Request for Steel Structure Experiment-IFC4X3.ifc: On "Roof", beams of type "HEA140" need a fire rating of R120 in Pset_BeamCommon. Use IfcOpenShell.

First a look at what the model holds.

```python
import ifcopenshell
import ifcopenshell.util.element

model = ifcopenshell.open("Steel Structure Experiment-IFC4X3.ifc")
print(model.schema)
storey = next(s for s in model.by_type("IfcBuildingStorey") if s.Name == "Roof")
beams = [e for e in ifcopenshell.util.element.get_decomposition(storey) if e.is_a("IfcBeam")]
seen = {}
for e in beams:
    element_type = ifcopenshell.util.element.get_type(e)
    key = (element_type.Name if element_type != e and element_type else None, ifcopenshell.util.element.get_pset(e, "Pset_BeamCommon", "FireRating"))
    seen[key] = seen.get(key, 0) + 1
for (name, value), count in sorted(seen.items(), key=str):
    print(count, "x", name, "|", value)
```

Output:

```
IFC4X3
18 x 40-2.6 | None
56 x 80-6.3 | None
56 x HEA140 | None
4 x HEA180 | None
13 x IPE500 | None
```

```python
import ifcopenshell
import ifcopenshell.api.pset
import ifcopenshell.util.element

model = ifcopenshell.open("Steel Structure Experiment-IFC4X3.ifc")

storey = next(s for s in model.by_type("IfcBuildingStorey") if s.Name == "Roof")
beams = [e for e in ifcopenshell.util.element.get_decomposition(storey) if e.is_a("IfcBeam")]

count = 0
for e in beams:
    element_type = ifcopenshell.util.element.get_type(e)
    if element_type in (None, e) or element_type.Name != "HEA140":
        continue
    # add_pset returns the element's existing set when there is one.
    pset = ifcopenshell.api.pset.add_pset(model, product=e, name="Pset_BeamCommon")
    ifcopenshell.api.pset.edit_pset(model, pset=pset, properties={"FireRating": "R120"})
    count += 1

print(count, "beams updated")

model.write("Steel Structure Experiment-IFC4X3_edited.ifc")
```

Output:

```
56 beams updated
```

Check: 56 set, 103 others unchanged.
